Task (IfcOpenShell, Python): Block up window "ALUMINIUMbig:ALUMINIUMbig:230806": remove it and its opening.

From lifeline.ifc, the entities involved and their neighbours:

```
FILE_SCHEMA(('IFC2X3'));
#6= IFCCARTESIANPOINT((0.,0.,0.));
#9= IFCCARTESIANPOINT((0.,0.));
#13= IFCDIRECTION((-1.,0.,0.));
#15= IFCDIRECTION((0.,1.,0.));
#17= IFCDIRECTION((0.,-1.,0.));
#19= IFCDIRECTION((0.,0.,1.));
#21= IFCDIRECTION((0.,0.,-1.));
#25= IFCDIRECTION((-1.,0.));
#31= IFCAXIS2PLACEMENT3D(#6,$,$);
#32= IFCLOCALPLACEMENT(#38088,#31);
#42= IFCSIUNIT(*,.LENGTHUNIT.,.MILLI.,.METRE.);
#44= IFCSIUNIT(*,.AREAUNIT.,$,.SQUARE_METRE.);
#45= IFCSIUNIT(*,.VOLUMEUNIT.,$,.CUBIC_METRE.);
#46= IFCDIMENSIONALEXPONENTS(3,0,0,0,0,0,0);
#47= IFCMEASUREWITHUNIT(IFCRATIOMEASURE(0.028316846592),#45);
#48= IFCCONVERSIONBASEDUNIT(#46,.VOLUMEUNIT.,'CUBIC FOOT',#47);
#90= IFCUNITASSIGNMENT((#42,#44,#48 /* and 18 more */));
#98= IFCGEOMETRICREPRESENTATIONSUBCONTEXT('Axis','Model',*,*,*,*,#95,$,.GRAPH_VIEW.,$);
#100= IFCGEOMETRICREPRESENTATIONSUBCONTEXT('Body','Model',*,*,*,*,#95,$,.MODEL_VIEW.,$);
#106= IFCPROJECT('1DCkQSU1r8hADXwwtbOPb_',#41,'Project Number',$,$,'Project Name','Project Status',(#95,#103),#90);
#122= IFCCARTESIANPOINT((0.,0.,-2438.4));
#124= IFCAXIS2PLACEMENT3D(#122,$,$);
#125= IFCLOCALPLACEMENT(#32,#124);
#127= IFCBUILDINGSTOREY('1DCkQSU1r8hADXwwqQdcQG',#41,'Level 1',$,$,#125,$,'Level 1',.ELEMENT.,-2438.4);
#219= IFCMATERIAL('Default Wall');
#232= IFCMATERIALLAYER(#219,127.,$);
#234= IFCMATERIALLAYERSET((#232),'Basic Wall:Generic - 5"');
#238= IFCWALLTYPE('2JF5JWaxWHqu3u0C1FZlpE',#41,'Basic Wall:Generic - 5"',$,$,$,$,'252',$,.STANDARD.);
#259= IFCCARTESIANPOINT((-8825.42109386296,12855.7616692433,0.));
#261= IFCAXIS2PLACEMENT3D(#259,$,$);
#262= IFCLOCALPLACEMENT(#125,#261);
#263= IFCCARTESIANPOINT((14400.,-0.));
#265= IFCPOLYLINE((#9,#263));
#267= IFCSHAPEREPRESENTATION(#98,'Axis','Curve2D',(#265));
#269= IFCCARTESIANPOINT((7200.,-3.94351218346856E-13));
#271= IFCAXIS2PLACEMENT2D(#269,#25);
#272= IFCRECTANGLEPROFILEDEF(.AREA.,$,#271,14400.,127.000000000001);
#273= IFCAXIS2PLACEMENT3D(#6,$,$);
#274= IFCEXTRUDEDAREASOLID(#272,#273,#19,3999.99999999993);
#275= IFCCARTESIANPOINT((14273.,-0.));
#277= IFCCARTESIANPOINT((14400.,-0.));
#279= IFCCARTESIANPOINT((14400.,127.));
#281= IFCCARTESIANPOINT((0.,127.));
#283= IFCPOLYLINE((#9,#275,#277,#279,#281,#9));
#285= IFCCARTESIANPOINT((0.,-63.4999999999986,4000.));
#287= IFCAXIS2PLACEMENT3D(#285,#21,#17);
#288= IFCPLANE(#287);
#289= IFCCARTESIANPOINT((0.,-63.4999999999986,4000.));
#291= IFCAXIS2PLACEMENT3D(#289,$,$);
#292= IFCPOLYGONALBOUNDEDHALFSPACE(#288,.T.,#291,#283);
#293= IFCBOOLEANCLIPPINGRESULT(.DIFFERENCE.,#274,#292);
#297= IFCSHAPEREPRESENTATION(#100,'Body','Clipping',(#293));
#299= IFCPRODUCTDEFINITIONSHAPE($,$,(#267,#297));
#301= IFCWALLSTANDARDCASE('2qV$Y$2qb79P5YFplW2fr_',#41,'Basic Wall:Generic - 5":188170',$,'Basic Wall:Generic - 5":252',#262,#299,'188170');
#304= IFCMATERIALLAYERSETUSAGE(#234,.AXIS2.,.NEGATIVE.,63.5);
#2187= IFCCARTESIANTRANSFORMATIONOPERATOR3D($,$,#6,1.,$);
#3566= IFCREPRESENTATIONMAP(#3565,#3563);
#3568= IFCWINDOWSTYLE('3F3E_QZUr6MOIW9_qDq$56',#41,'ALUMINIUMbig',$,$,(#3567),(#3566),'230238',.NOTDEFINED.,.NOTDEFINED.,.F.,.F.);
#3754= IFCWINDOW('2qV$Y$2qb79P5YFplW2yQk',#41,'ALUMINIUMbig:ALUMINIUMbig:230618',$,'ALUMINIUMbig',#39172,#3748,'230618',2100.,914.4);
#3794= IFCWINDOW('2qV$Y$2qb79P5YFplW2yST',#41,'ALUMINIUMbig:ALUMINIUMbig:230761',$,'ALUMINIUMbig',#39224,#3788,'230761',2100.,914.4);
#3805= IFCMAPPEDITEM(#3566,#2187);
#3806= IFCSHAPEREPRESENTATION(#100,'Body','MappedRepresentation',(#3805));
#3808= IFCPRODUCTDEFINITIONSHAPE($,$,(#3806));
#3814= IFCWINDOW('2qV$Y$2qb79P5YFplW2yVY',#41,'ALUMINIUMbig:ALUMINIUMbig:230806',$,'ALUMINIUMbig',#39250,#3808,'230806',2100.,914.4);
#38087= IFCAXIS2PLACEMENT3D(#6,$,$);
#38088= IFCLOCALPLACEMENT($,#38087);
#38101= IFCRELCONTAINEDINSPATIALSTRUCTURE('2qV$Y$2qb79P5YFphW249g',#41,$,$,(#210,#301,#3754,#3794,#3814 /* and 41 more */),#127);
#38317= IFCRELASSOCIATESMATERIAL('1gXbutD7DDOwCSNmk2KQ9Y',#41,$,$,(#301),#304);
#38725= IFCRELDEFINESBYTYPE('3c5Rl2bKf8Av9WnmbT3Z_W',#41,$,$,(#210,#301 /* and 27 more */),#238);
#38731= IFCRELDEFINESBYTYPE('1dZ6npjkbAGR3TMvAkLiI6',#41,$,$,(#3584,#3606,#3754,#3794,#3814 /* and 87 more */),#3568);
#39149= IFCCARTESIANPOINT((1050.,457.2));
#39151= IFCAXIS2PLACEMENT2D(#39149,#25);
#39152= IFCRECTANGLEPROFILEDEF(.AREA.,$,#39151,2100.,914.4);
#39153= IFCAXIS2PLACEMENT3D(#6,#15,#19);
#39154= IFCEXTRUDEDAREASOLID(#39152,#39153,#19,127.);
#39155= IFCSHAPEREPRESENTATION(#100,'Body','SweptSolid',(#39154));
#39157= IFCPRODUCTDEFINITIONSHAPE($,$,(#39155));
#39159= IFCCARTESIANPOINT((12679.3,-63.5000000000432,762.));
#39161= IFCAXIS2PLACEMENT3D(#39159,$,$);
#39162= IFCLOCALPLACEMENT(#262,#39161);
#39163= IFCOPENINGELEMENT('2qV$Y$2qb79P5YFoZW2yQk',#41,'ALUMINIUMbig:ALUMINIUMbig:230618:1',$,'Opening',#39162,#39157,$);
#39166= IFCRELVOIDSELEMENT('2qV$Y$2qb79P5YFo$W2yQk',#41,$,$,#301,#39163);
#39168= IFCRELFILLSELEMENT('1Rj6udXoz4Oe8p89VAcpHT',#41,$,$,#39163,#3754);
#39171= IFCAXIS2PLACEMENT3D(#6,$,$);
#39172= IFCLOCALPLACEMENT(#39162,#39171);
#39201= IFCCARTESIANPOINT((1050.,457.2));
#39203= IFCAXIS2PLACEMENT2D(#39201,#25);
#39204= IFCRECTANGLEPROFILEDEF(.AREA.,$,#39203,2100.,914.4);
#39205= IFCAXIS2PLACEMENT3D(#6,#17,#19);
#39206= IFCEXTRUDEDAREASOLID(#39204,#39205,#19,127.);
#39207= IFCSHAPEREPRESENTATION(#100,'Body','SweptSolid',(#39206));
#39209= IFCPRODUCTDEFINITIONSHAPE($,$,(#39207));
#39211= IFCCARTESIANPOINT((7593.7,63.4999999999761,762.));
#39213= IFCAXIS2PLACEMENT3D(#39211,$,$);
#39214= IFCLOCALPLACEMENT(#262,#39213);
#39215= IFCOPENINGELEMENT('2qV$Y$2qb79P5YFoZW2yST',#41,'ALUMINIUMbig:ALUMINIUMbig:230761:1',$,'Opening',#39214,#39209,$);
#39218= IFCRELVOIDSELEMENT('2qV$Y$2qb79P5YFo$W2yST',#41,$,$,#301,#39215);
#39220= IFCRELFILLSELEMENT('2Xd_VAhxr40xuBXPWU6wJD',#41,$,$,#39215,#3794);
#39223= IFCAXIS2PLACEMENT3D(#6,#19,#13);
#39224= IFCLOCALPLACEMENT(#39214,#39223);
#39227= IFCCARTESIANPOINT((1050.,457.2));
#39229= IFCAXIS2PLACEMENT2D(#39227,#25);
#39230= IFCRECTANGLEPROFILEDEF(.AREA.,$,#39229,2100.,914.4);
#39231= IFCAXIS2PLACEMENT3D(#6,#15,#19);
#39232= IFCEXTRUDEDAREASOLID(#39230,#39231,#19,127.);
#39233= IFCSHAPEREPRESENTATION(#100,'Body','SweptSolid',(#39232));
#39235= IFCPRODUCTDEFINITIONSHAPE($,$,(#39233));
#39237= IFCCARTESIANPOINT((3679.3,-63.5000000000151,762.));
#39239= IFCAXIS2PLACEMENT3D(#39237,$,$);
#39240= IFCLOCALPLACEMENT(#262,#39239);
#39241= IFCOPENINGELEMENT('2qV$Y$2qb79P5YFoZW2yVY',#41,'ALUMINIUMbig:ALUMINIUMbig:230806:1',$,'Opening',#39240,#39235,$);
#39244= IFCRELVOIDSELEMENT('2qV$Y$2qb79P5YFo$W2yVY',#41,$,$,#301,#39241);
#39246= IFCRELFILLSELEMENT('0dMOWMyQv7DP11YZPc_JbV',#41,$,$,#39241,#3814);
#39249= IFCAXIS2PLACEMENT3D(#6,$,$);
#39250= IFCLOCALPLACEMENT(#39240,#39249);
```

```python
import ifcopenshell
import ifcopenshell.api.feature
import ifcopenshell.api.root
import ifcopenshell.geom
import ifcopenshell.util.shape

model = ifcopenshell.open("lifeline.ifc")
settings = ifcopenshell.geom.settings()


def volume(element):
    """Net volume in cubic metres, openings subtracted."""
    shape = ifcopenshell.geom.create_shape(settings, element)
    return ifcopenshell.util.shape.get_volume(shape.geometry)


window = model.by_guid("2qV$Y$2qb79P5YFplW2yVY")
opening = window.FillsVoids[0].RelatingOpeningElement
wall = opening.VoidsElements[0].RelatingBuildingElement
before = volume(wall)

ifcopenshell.api.root.remove_product(model, product=window)
ifcopenshell.api.feature.remove_feature(model, feature=opening)

after = volume(wall)

print(f"wall volume {before:.3f} -> {after:.3f} m3")

model.write("lifeline_updated.ifc")
```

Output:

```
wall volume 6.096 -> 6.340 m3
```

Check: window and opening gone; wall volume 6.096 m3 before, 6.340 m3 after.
